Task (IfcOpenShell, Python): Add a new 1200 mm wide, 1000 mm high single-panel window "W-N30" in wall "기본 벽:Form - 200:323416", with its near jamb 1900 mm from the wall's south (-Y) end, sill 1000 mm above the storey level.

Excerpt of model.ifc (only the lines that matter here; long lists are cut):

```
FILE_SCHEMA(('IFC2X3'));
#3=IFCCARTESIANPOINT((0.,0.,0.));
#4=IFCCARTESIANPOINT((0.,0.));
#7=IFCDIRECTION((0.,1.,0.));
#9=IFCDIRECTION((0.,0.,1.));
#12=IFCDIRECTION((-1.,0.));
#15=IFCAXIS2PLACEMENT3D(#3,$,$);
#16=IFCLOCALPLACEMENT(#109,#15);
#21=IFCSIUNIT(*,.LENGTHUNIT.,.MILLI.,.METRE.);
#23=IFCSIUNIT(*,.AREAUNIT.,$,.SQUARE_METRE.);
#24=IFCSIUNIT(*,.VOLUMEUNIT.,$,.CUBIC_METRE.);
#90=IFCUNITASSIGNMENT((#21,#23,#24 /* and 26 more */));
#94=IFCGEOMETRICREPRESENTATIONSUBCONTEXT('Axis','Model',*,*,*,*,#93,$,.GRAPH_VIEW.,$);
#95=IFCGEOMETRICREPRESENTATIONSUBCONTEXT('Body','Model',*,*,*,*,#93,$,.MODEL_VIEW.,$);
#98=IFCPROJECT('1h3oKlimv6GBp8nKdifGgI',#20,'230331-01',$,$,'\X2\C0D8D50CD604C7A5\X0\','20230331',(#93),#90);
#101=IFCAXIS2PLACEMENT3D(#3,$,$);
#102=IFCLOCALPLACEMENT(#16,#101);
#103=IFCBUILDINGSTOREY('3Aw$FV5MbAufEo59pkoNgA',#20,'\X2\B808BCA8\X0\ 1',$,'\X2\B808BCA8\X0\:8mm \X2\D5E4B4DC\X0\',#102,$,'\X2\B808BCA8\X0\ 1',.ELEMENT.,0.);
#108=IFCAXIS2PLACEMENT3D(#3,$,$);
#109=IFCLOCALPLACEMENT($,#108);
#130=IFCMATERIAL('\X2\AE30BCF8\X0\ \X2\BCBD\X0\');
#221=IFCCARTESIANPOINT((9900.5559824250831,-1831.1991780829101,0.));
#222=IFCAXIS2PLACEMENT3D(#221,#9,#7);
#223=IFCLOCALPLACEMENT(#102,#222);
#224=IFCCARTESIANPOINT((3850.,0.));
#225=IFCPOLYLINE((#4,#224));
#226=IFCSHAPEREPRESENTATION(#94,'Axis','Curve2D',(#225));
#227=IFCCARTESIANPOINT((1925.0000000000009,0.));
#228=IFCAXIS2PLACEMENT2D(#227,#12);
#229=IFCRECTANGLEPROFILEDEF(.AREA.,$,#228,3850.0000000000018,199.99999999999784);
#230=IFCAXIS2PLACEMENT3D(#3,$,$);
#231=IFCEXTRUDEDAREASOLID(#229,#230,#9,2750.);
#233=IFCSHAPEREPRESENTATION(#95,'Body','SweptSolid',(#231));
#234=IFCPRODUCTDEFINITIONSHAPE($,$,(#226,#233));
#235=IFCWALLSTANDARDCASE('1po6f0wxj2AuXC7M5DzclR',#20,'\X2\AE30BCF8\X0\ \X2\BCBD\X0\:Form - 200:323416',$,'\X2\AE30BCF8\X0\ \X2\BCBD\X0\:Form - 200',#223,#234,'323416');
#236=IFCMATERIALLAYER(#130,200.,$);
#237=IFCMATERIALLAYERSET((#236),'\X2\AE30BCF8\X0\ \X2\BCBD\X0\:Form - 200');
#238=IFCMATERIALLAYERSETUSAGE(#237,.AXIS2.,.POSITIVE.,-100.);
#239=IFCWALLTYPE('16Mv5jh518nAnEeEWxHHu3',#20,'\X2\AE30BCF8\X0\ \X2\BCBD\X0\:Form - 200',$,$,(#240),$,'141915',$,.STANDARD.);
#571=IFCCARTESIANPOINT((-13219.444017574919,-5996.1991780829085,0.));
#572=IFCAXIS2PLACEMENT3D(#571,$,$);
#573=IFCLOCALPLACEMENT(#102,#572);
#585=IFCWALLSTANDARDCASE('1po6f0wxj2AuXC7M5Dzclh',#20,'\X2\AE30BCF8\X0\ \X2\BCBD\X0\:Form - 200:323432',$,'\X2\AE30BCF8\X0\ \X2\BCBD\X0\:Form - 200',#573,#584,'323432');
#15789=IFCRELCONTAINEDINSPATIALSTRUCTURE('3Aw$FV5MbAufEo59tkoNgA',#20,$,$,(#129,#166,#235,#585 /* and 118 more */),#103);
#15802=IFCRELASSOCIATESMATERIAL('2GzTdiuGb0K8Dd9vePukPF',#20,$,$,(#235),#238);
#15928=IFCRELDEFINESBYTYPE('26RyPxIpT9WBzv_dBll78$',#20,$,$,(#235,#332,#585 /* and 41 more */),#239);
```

```python
import numpy as np
import ifcopenshell
import ifcopenshell.api.feature
import ifcopenshell.api.geometry
import ifcopenshell.api.root
import ifcopenshell.api.spatial
import ifcopenshell.api.type
import ifcopenshell.geom
import ifcopenshell.util.element
import ifcopenshell.util.placement
import ifcopenshell.util.representation
import ifcopenshell.util.shape
import ifcopenshell.util.unit

model = ifcopenshell.open("model.ifc")
unit_scale = ifcopenshell.util.unit.calculate_unit_scale(model)
settings = ifcopenshell.geom.settings()


def volume(element):
    """Net volume in cubic metres, openings subtracted."""
    shape = ifcopenshell.geom.create_shape(settings, element)
    return ifcopenshell.util.shape.get_volume(shape.geometry)


wall = model.by_guid("1po6f0wxj2AuXC7M5DzclR")
storey = ifcopenshell.util.element.get_container(wall, ifc_class="IfcBuildingStorey")
context = ifcopenshell.util.representation.get_context(model, "Model", "Body", "MODEL_VIEW")
before = volume(wall)

width, height, from_end, sill = 1.2, 1, 1.9, 1  # metres

# The wall runs along its own X axis, and the end named is its -X end.
wall_shape = ifcopenshell.geom.create_shape(settings, wall)
x, y, z = ifcopenshell.util.shape.get_vertices(wall_shape.geometry).T
start = x.min() + from_end
face, thickness = float(y.min()), float(y.max() - y.min())
wall_matrix = ifcopenshell.util.placement.get_local_placement(wall.ObjectPlacement)
level = ifcopenshell.util.placement.get_local_placement(storey.ObjectPlacement)[2, 3]


def in_wall(x, y):
    """Placement at x, y metres in the wall's axes, at sill height."""
    matrix = wall_matrix.copy()
    matrix[:, 3] = wall_matrix @ np.array([x / unit_scale, y / unit_scale, 0.0, 1.0])
    matrix[2, 3] = level + sill / unit_scale
    return matrix


# Opening: a box that overshoots both wall faces by 50 mm.
opening = ifcopenshell.api.root.create_entity(model, ifc_class="IfcOpeningElement")
box = ifcopenshell.api.geometry.add_wall_representation(
    model, context=context, length=width, height=height, thickness=thickness + 0.1
)
ifcopenshell.api.geometry.assign_representation(model, product=opening, representation=box)
ifcopenshell.api.geometry.edit_object_placement(model, product=opening, matrix=in_wall(start, face - 0.05), is_si=False)
ifcopenshell.api.feature.add_feature(model, feature=opening, element=wall)

window = ifcopenshell.api.root.create_entity(model, ifc_class="IfcWindow", name="W-N30")
window.OverallWidth, window.OverallHeight = width / unit_scale, height / unit_scale
body = ifcopenshell.api.geometry.add_window_representation(
    model,
    context=context,
    overall_width=window.OverallWidth,
    overall_height=window.OverallHeight,
    partition_type="SINGLE_PANEL",
)
ifcopenshell.api.geometry.assign_representation(model, product=window, representation=body)
ifcopenshell.api.spatial.assign_container(model, products=[window], relating_structure=storey)
fills = ifcopenshell.api.feature.add_filling(model, opening=opening, element=window)
fills.OwnerHistory = window.OwnerHistory  # required in IFC2X3

# IFC2X3 keeps the operation on the window style.
style = ifcopenshell.api.root.create_entity(model, ifc_class="IfcWindowStyle", name="W-N30")
style.OperationType, style.ConstructionType = "SINGLE_PANEL", "NOTDEFINED"
style.ParameterTakesPrecedence = style.Sizeable = False
ifcopenshell.api.type.assign_type(model, related_objects=[window], relating_type=style)

# Centre the window in the wall's thickness.
ifcopenshell.api.geometry.edit_object_placement(model, product=window, matrix=in_wall(start, face), is_si=False)
window_shape = ifcopenshell.geom.create_shape(settings, window)
depth = ifcopenshell.util.shape.get_vertices(window_shape.geometry)[:, 1]
offset = face + thickness / 2 - (depth.min() + depth.max()) / 2
ifcopenshell.api.geometry.edit_object_placement(model, product=window, matrix=in_wall(start, offset), is_si=False)

after = volume(wall)

print(f"wall volume {before:.3f} -> {after:.3f} m3")

model.write("model_updated.ifc")
```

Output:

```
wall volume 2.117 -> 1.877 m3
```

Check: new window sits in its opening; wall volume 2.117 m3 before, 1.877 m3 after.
